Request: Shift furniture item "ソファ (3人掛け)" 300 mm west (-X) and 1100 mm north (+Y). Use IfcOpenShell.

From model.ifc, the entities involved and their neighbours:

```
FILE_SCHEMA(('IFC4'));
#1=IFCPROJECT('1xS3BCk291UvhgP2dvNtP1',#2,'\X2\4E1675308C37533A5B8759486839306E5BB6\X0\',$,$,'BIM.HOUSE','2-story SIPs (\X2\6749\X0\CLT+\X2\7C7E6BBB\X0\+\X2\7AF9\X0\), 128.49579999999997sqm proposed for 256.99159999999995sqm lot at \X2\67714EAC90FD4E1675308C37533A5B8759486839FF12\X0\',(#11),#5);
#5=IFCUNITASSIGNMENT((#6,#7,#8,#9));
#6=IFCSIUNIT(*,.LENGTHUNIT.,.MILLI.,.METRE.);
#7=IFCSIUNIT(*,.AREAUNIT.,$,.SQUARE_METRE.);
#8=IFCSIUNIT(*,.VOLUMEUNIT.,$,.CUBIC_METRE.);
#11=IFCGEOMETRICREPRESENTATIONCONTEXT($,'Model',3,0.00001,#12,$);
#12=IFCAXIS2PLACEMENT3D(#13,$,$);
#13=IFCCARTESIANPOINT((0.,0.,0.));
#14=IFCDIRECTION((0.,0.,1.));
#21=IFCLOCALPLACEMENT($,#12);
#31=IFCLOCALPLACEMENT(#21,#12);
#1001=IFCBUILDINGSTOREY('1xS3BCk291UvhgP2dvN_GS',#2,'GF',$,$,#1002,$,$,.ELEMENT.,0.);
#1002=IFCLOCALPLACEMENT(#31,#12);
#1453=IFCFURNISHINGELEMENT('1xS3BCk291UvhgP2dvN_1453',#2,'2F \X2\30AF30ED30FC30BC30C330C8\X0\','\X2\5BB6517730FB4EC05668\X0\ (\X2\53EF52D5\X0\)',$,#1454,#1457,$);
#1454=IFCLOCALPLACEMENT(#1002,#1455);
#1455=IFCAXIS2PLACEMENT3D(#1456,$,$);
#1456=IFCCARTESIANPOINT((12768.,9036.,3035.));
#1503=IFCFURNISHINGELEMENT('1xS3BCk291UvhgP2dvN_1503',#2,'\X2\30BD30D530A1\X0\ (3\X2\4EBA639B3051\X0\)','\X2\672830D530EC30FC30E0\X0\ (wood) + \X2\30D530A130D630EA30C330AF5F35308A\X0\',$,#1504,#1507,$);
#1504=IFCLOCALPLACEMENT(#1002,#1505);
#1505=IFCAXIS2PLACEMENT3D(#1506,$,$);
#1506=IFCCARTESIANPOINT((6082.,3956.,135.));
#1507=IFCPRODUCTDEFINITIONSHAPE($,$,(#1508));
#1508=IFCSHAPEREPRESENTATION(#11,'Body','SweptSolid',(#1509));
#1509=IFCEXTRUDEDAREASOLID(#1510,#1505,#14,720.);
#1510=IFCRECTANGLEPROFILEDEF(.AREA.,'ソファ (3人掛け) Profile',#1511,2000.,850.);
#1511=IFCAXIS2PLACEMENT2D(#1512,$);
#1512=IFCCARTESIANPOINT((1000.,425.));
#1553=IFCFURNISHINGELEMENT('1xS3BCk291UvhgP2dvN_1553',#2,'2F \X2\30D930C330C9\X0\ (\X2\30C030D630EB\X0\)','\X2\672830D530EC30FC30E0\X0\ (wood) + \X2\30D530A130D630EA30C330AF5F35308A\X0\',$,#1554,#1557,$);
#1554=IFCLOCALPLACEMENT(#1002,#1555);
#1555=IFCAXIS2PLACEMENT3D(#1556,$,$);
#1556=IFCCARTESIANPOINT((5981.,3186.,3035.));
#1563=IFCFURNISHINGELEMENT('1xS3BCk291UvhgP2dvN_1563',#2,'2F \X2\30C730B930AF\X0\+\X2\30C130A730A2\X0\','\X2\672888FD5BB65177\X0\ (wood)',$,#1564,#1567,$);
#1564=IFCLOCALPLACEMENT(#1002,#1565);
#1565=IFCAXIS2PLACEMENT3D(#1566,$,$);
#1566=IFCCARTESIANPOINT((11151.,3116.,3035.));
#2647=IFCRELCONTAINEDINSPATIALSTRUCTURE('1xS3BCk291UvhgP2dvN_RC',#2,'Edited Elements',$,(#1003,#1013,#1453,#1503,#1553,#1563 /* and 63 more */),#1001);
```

```python
import ifcopenshell
import ifcopenshell.api.geometry
import ifcopenshell.util.placement

model = ifcopenshell.open("model.ifc")

item = model.by_id(1503)
matrix = ifcopenshell.util.placement.get_local_placement(item.ObjectPlacement)
matrix[0, 3] -= 300.0
matrix[1, 3] += 1100.0
ifcopenshell.api.geometry.edit_object_placement(model, product=item, matrix=matrix, is_si=False)

print(ifcopenshell.util.placement.get_local_placement(item.ObjectPlacement).round(3) + 0.0)

model.write("model_rev.ifc")
```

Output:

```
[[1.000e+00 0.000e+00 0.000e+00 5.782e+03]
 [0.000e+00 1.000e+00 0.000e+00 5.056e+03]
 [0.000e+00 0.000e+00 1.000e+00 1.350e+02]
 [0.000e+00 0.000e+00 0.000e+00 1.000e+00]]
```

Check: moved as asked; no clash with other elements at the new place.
